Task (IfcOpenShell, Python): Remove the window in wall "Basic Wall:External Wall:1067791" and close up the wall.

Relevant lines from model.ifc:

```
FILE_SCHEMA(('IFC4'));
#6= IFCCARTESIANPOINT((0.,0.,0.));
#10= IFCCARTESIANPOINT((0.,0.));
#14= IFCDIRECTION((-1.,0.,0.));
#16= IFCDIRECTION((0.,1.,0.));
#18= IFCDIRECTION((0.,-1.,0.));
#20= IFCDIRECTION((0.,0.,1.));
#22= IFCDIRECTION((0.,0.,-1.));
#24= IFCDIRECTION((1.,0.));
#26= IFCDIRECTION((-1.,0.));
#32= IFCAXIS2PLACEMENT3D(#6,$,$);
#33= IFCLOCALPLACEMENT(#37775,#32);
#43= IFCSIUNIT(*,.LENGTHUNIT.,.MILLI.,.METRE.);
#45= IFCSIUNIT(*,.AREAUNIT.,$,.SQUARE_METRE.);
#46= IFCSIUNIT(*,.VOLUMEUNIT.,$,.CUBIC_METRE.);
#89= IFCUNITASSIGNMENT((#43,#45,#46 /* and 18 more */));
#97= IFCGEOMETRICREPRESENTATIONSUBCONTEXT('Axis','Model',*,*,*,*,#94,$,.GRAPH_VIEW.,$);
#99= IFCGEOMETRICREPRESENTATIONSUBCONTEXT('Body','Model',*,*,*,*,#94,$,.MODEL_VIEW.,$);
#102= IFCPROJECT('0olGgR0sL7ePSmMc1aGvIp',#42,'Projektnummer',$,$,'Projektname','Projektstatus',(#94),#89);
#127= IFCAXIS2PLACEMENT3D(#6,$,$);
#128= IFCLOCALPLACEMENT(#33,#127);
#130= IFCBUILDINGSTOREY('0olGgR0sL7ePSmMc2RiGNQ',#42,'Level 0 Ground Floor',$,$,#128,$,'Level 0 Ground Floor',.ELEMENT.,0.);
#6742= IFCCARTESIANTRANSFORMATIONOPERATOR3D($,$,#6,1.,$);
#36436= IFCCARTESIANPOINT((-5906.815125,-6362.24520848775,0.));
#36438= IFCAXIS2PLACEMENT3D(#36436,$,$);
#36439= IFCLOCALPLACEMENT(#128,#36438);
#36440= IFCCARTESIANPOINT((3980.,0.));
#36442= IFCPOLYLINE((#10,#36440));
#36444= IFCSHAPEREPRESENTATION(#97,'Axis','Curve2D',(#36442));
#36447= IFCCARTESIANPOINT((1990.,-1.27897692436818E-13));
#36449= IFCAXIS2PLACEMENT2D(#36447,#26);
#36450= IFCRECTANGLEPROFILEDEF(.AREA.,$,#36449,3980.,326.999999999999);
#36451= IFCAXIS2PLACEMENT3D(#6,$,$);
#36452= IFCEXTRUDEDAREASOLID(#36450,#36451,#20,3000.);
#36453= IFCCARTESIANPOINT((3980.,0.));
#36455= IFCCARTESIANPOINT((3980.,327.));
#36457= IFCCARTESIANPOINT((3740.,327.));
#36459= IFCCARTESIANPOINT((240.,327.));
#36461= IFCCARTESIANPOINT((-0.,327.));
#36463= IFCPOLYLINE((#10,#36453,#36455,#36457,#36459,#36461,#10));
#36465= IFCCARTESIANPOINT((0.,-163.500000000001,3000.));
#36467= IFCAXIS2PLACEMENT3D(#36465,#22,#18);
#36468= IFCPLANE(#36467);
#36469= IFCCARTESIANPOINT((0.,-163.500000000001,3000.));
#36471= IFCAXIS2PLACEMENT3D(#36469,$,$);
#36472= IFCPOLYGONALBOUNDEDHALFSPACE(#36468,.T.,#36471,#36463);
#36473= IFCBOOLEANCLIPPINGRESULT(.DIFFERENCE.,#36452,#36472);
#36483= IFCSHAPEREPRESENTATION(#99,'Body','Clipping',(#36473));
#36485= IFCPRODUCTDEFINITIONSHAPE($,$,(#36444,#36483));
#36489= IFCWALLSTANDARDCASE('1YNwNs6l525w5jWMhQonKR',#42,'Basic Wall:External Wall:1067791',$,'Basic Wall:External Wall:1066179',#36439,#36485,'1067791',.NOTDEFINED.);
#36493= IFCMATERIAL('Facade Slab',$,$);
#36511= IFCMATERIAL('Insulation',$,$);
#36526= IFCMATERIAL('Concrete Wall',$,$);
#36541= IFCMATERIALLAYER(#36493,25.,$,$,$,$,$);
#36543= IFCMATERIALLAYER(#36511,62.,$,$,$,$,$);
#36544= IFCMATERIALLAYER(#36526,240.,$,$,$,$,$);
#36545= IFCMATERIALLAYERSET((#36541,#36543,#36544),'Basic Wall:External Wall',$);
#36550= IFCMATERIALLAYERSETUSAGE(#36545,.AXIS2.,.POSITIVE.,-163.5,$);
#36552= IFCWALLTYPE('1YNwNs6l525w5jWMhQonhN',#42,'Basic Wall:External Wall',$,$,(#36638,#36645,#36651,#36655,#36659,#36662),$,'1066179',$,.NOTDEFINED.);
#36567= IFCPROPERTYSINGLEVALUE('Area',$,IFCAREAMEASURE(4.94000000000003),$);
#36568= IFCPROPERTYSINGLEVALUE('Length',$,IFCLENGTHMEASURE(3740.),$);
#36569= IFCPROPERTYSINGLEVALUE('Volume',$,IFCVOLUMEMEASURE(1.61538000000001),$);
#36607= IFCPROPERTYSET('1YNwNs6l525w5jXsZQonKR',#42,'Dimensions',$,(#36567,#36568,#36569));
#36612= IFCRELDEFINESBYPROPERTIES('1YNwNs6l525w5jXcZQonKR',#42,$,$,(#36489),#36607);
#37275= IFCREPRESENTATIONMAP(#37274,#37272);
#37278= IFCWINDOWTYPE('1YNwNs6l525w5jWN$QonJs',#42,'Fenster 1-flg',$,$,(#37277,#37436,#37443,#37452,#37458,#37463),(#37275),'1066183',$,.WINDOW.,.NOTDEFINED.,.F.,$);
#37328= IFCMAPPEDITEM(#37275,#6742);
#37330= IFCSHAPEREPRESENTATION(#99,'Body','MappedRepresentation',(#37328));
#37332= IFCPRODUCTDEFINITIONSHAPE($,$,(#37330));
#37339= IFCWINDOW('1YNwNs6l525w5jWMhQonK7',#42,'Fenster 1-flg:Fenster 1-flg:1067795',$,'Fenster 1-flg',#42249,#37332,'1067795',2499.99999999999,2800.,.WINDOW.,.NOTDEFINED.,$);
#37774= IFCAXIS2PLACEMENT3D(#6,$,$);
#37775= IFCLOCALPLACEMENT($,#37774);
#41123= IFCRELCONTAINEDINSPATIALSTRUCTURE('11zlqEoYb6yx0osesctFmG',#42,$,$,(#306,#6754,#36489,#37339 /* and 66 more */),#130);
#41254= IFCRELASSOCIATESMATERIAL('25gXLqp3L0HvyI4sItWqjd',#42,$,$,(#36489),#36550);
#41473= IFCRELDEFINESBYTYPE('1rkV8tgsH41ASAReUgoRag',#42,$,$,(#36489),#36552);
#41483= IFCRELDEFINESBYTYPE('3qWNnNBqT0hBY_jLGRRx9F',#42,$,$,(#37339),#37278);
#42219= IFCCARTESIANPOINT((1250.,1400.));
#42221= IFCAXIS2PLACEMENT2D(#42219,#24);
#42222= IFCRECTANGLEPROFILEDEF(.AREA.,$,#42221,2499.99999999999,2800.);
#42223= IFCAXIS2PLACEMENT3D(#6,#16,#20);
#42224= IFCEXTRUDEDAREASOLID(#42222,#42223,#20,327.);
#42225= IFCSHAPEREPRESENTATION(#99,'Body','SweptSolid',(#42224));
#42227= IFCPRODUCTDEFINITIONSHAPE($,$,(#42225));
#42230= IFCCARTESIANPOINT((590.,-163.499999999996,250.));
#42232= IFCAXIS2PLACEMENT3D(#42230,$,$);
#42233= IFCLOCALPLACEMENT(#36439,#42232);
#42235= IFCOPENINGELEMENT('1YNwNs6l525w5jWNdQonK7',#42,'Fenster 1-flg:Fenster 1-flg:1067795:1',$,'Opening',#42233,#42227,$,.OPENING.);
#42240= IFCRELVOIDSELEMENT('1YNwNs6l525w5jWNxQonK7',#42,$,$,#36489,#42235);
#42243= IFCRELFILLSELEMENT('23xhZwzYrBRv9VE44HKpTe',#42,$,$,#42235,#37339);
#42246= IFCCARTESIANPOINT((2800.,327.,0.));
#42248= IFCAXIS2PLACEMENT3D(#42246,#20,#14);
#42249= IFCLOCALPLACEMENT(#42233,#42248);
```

```python
import ifcopenshell
import ifcopenshell.api.feature
import ifcopenshell.api.pset
import ifcopenshell.api.root
import ifcopenshell.geom
import ifcopenshell.util.element
import ifcopenshell.util.shape
import ifcopenshell.util.unit

model = ifcopenshell.open("model.ifc")
area_scale = ifcopenshell.util.unit.calculate_unit_scale(model, "AREAUNIT")
volume_scale = ifcopenshell.util.unit.calculate_unit_scale(model, "VOLUMEUNIT")
settings = ifcopenshell.geom.settings()


def volume(element):
    """Net volume in cubic metres, openings subtracted."""
    shape = ifcopenshell.geom.create_shape(settings, element)
    return ifcopenshell.util.shape.get_volume(shape.geometry)


window = model.by_guid("1YNwNs6l525w5jWMhQonK7")
opening = window.FillsVoids[0].RelatingOpeningElement
wall = opening.VoidsElements[0].RelatingBuildingElement
before = volume(wall)

ifcopenshell.api.root.remove_product(model, product=window)
ifcopenshell.api.feature.remove_feature(model, feature=opening)

after = volume(wall)
thickness = 0.327  # wall thickness in metres

# Update the wall's stored quantities.
pset = model.by_id(ifcopenshell.util.element.get_pset(wall, "Dimensions", should_inherit=False)["id"])
ifcopenshell.api.pset.edit_pset(model, pset=pset, properties={
    "Area": model.create_entity("IfcAreaMeasure", after / thickness / area_scale),
    "Volume": model.create_entity("IfcVolumeMeasure", after / volume_scale),
})

print(f"wall volume {before:.3f} -> {after:.3f} m3")

model.write("model_updated.ifc")
```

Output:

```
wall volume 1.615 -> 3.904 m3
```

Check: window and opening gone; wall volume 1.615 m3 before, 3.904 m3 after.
